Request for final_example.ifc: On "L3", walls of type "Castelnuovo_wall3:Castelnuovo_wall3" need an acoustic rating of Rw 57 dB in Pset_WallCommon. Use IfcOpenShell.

First a look at what the model holds.

```python
import ifcopenshell
import ifcopenshell.util.element

model = ifcopenshell.open("final_example.ifc")
print(model.schema)
storey = next(s for s in model.by_type("IfcBuildingStorey") if s.Name == "L3")
walls = [e for e in ifcopenshell.util.element.get_decomposition(storey) if e.is_a("IfcWall")]
seen = {}
for e in walls:
    element_type = ifcopenshell.util.element.get_type(e)
    key = (element_type.Name if element_type != e and element_type else None, ifcopenshell.util.element.get_pset(e, "Pset_WallCommon", "AcousticRating"))
    seen[key] = seen.get(key, 0) + 1
for (name, value), count in sorted(seen.items(), key=str):
    print(count, "x", name, "|", value)
```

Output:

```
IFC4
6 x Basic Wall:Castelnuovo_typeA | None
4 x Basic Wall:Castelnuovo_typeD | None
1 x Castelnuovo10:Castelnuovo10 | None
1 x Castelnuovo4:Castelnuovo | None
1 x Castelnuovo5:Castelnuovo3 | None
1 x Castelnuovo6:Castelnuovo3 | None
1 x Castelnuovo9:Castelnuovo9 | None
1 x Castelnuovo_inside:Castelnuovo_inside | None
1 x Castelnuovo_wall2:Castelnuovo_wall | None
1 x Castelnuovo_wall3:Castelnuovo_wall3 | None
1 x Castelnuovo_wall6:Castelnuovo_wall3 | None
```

```python
import ifcopenshell
import ifcopenshell.api.pset
import ifcopenshell.util.element

model = ifcopenshell.open("final_example.ifc")

storey = next(s for s in model.by_type("IfcBuildingStorey") if s.Name == "L3")
walls = [e for e in ifcopenshell.util.element.get_decomposition(storey) if e.is_a("IfcWall")]

count = 0
for e in walls:
    element_type = ifcopenshell.util.element.get_type(e)
    if element_type in (None, e) or element_type.Name != "Castelnuovo_wall3:Castelnuovo_wall3":
        continue
    # add_pset returns the element's existing set when there is one.
    pset = ifcopenshell.api.pset.add_pset(model, product=e, name="Pset_WallCommon")
    ifcopenshell.api.pset.edit_pset(model, pset=pset, properties={"AcousticRating": "Rw 57 dB"})
    count += 1

print(count, "walls updated")

model.write("final_example_updated.ifc")
```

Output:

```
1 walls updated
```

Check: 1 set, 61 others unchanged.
